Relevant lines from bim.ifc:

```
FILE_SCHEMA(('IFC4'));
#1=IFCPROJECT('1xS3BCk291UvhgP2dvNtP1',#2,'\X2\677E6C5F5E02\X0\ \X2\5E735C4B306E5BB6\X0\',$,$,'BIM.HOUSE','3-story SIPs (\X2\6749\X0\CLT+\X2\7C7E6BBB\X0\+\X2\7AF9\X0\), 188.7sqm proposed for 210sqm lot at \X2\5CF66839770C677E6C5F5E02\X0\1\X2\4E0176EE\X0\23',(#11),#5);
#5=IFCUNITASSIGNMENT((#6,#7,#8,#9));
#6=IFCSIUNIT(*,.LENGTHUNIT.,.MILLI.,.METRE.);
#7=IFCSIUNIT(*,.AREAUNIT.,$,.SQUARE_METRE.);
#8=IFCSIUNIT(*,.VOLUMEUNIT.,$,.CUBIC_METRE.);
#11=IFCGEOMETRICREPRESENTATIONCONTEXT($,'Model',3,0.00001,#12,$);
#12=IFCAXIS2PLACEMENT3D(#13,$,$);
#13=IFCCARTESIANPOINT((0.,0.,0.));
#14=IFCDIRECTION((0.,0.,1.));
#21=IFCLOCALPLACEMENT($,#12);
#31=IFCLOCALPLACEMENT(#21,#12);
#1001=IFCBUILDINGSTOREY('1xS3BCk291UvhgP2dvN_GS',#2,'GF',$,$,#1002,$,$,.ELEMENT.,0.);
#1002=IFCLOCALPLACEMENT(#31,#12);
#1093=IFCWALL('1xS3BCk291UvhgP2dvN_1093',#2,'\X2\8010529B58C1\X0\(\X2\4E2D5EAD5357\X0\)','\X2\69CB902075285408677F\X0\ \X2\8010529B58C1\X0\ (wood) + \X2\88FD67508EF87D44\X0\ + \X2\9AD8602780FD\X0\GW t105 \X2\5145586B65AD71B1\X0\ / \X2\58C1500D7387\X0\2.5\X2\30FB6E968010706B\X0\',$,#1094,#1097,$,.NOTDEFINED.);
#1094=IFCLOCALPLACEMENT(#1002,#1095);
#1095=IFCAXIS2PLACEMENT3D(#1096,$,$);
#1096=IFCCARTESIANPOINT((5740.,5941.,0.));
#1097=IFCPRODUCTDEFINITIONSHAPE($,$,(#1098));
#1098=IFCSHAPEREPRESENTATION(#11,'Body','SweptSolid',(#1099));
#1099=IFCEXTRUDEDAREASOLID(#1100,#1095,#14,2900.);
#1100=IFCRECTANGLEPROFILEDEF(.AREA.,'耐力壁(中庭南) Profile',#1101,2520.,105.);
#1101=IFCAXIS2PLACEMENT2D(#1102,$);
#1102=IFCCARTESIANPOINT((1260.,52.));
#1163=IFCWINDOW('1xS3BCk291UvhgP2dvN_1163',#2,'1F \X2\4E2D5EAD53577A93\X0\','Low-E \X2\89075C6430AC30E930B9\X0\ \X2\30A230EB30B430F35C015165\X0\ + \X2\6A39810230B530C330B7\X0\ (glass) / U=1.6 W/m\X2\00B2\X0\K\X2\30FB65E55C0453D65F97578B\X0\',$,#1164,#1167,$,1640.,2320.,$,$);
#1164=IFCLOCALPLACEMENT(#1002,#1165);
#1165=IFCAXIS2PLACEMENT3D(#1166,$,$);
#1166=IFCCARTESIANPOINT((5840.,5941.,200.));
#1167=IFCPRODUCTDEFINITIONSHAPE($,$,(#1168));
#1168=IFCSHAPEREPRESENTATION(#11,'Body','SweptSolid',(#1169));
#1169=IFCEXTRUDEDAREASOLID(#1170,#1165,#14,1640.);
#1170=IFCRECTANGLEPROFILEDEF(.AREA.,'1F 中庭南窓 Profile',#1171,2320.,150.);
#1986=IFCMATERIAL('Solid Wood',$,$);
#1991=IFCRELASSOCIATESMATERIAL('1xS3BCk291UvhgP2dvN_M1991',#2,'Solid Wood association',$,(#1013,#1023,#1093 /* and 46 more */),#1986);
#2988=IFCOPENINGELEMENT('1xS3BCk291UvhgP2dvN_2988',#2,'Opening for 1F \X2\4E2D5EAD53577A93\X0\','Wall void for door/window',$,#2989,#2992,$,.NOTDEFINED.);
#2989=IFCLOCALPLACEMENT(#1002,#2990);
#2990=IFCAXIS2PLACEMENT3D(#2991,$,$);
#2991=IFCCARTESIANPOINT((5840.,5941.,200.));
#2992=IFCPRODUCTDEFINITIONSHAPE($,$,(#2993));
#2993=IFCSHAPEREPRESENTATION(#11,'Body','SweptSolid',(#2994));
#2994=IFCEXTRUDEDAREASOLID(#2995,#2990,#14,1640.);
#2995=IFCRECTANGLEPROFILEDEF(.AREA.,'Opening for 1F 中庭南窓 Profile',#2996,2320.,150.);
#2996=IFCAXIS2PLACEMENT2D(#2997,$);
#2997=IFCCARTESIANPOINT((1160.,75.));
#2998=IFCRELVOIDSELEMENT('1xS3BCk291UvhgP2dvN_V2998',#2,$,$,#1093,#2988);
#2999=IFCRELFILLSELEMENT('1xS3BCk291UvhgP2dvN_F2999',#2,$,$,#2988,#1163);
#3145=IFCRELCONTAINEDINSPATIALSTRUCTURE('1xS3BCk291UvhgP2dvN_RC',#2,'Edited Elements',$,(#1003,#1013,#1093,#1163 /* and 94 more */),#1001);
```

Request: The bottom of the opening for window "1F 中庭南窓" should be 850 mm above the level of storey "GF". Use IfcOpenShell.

```python
import numpy as np
import ifcopenshell
import ifcopenshell.api.geometry
import ifcopenshell.geom
import ifcopenshell.util.element
import ifcopenshell.util.placement
import ifcopenshell.util.shape
import ifcopenshell.util.unit

model = ifcopenshell.open("bim.ifc")
unit_scale = ifcopenshell.util.unit.calculate_unit_scale(model)

window = model.by_guid("1xS3BCk291UvhgP2dvN_1163")
opening = window.FillsVoids[0].RelatingOpeningElement
storey = ifcopenshell.util.element.get_container(window, ifc_class="IfcBuildingStorey")
level = ifcopenshell.util.placement.get_local_placement(storey.ObjectPlacement)[2, 3]

# The opening's origin need not be at the sill, so measure its lowest point.
shape = ifcopenshell.geom.create_shape(ifcopenshell.geom.settings(), opening)
bottom = ifcopenshell.util.shape.get_shape_bottom_elevation(shape, shape.geometry) / unit_scale
dz = level + 850.0 - bottom

shift = np.array([0.0, 0.0, dz])
# The window is not placed relative to its opening, so move both.
for product in (opening, window):
    matrix = ifcopenshell.util.placement.get_local_placement(product.ObjectPlacement)
    matrix[:3, 3] += shift
    ifcopenshell.api.geometry.edit_object_placement(model, product=product, matrix=matrix, is_si=False)

print(f"moved by {dz * unit_scale:+.3f} m")

model.write("bim_v2.ifc")
```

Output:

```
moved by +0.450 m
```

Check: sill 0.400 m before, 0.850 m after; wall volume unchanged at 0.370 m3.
